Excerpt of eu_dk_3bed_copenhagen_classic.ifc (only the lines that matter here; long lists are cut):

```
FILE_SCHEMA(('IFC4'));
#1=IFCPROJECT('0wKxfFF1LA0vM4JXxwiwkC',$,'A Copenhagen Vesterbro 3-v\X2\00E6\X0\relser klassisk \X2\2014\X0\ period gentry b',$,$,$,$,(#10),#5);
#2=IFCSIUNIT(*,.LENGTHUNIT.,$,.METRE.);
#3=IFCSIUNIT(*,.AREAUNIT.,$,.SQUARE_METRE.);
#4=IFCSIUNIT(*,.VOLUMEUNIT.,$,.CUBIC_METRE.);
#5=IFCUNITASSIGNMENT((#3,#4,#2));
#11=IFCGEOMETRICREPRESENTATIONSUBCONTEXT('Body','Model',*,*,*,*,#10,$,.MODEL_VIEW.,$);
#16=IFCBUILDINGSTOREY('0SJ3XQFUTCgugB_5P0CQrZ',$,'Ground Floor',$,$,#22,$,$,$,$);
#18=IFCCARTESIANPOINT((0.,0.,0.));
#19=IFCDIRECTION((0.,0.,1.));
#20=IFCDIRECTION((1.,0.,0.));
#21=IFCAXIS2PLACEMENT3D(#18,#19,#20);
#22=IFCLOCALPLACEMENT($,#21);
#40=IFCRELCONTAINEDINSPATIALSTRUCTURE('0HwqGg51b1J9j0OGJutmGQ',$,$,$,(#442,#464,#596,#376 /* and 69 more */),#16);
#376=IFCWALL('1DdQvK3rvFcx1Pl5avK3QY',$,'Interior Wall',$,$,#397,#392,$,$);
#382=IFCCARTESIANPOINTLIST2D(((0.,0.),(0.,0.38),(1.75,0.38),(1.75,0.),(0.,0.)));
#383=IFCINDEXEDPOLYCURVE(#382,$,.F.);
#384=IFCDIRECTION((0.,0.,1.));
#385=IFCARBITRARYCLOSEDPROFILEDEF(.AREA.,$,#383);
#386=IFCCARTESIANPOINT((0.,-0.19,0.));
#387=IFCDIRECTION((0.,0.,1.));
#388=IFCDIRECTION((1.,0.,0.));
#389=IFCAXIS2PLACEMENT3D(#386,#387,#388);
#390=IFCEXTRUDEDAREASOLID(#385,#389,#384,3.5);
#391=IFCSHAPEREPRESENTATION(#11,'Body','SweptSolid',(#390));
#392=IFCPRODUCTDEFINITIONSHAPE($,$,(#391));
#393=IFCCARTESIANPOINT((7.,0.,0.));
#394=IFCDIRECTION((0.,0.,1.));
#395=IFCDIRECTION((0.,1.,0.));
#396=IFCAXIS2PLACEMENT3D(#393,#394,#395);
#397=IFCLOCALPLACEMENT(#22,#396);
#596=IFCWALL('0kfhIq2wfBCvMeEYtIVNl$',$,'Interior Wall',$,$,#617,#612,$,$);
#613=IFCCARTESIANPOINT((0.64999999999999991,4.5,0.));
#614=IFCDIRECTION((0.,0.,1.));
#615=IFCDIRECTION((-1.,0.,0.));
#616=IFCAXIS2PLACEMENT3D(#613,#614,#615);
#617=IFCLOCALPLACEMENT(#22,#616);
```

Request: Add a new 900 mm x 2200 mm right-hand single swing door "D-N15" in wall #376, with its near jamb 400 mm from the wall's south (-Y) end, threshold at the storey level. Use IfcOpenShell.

```python
import numpy as np
import ifcopenshell
import ifcopenshell.api.feature
import ifcopenshell.api.geometry
import ifcopenshell.api.root
import ifcopenshell.api.spatial
import ifcopenshell.geom
import ifcopenshell.util.element
import ifcopenshell.util.placement
import ifcopenshell.util.representation
import ifcopenshell.util.shape
import ifcopenshell.util.unit

model = ifcopenshell.open("eu_dk_3bed_copenhagen_classic.ifc")
unit_scale = ifcopenshell.util.unit.calculate_unit_scale(model)
settings = ifcopenshell.geom.settings()


def volume(element):
    """Net volume in cubic metres, openings subtracted."""
    shape = ifcopenshell.geom.create_shape(settings, element)
    return ifcopenshell.util.shape.get_volume(shape.geometry)


wall = model.by_id(376)
storey = ifcopenshell.util.element.get_container(wall, ifc_class="IfcBuildingStorey")
context = ifcopenshell.util.representation.get_context(model, "Model", "Body", "MODEL_VIEW")
before = volume(wall)

width, height, from_end, sill = 0.9, 2.2, 0.4, 0.0  # metres

# The wall runs along its own X axis, and the end named is its -X end.
wall_shape = ifcopenshell.geom.create_shape(settings, wall)
x, y, z = ifcopenshell.util.shape.get_vertices(wall_shape.geometry).T
start = x.min() + from_end
face, thickness = float(y.min()), float(y.max() - y.min())
wall_matrix = ifcopenshell.util.placement.get_local_placement(wall.ObjectPlacement)
level = ifcopenshell.util.placement.get_local_placement(storey.ObjectPlacement)[2, 3]


def in_wall(x, y):
    """Placement at x, y metres in the wall's axes, at sill height."""
    matrix = wall_matrix.copy()
    matrix[:, 3] = wall_matrix @ np.array([x / unit_scale, y / unit_scale, 0.0, 1.0])
    matrix[2, 3] = level + sill / unit_scale
    return matrix


# Opening: a box that overshoots both wall faces by 50 mm.
opening = ifcopenshell.api.root.create_entity(model, ifc_class="IfcOpeningElement", predefined_type="OPENING")
box = ifcopenshell.api.geometry.add_wall_representation(
    model, context=context, length=width, height=height, thickness=thickness + 0.1
)
ifcopenshell.api.geometry.assign_representation(model, product=opening, representation=box)
ifcopenshell.api.geometry.edit_object_placement(model, product=opening, matrix=in_wall(start, face - 0.05), is_si=False)
ifcopenshell.api.feature.add_feature(model, feature=opening, element=wall)

door = ifcopenshell.api.root.create_entity(model, ifc_class="IfcDoor", name="D-N15", predefined_type="DOOR")
door.OverallWidth, door.OverallHeight = width / unit_scale, height / unit_scale
door.OperationType = "SINGLE_SWING_RIGHT"
body = ifcopenshell.api.geometry.add_door_representation(
    model,
    context=context,
    overall_width=door.OverallWidth,
    overall_height=door.OverallHeight,
    operation_type="SINGLE_SWING_RIGHT",
    lining_properties={"LiningDepth": thickness / unit_scale, "ThresholdDepth": thickness / unit_scale},
)
ifcopenshell.api.geometry.assign_representation(model, product=door, representation=body)
ifcopenshell.api.spatial.assign_container(model, products=[door], relating_structure=storey)
ifcopenshell.api.feature.add_filling(model, opening=opening, element=door)

# The lining spans the wall, so the door starts at the wall face.
ifcopenshell.api.geometry.edit_object_placement(model, product=door, matrix=in_wall(start, face), is_si=False)

after = volume(wall)

print(f"wall volume {before:.3f} -> {after:.3f} m3")

model.write("eu_dk_3bed_copenhagen_classic_edited.ifc")
```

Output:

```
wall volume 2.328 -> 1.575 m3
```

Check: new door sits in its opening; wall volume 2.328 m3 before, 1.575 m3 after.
